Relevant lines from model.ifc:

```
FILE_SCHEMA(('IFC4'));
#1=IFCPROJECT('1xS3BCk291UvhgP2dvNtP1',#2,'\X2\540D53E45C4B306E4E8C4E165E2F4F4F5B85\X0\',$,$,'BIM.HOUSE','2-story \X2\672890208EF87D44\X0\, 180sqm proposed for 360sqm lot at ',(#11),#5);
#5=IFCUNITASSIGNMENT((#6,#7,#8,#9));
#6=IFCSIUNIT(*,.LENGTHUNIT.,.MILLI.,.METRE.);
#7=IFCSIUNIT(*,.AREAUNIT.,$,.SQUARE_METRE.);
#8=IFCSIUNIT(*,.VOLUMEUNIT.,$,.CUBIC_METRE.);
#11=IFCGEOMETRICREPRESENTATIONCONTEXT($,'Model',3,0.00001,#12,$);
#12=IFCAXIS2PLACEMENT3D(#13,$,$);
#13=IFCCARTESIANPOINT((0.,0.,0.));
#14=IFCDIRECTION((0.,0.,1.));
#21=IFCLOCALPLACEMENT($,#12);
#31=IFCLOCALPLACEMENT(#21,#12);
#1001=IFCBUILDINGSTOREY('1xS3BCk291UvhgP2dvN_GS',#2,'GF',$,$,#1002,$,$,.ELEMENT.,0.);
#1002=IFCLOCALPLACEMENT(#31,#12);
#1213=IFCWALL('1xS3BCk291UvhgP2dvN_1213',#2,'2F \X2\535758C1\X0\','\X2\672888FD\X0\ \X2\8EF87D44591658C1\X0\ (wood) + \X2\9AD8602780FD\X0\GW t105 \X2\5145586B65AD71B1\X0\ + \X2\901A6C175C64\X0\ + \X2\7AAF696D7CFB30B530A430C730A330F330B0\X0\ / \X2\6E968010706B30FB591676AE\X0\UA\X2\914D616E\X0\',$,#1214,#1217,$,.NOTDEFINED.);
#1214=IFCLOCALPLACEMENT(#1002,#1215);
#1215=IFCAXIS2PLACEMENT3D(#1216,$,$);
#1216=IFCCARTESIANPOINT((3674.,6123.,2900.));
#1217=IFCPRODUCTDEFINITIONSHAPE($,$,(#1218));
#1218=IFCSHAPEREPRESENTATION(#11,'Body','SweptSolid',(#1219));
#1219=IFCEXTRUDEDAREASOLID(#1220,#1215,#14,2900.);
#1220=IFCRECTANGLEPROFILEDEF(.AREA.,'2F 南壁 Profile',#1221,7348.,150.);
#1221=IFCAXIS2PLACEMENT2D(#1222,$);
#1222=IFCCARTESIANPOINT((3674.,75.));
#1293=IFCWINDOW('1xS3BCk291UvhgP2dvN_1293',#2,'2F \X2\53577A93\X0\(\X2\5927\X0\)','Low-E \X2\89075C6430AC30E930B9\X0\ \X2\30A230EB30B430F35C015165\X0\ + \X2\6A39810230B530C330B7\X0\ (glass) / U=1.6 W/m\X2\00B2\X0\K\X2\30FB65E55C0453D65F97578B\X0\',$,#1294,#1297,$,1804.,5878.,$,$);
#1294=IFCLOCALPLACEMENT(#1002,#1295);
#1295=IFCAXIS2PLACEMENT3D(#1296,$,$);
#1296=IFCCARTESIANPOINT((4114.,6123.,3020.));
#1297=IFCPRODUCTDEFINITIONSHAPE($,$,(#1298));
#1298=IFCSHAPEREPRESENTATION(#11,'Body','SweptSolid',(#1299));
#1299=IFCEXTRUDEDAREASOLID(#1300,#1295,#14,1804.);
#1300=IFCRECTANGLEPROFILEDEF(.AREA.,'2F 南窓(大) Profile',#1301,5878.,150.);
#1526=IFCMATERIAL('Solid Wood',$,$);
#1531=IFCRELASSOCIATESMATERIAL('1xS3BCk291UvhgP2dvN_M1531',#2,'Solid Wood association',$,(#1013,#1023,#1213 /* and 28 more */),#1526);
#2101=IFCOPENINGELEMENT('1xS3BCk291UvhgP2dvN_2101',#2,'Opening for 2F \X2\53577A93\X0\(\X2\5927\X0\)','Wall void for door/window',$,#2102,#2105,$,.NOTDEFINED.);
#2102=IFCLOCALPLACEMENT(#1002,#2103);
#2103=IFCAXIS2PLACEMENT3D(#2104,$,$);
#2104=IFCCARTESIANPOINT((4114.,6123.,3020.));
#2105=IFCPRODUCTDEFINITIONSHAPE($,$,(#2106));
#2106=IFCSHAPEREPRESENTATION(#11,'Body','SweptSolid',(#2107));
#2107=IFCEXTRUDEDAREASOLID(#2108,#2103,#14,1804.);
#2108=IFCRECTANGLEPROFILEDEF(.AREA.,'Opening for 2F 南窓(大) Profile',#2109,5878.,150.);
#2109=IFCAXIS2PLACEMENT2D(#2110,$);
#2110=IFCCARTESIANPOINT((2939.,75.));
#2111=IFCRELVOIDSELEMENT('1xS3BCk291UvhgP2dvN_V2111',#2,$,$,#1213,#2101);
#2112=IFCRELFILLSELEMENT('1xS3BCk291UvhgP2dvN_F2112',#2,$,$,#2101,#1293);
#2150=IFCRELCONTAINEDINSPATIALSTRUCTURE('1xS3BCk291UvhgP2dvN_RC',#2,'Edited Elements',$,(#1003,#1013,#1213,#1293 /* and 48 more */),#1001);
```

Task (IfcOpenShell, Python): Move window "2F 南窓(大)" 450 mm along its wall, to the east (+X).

```python
import ifcopenshell
import ifcopenshell.api.geometry
import ifcopenshell.util.placement

model = ifcopenshell.open("model.ifc")

window = model.by_id(1293)
opening = window.FillsVoids[0].RelatingOpeningElement
wall = opening.VoidsElements[0].RelatingBuildingElement

wall_matrix = ifcopenshell.util.placement.get_local_placement(wall.ObjectPlacement)
shift = wall_matrix[:3, 0] * 450.0
before = ifcopenshell.util.placement.get_local_placement(window.ObjectPlacement)[:3, 3].copy()

# The window is not placed relative to its opening, so move both.
for product in (opening, window):
    matrix = ifcopenshell.util.placement.get_local_placement(product.ObjectPlacement)
    matrix[:3, 3] += shift
    ifcopenshell.api.geometry.edit_object_placement(model, product=product, matrix=matrix, is_si=False)

after = ifcopenshell.util.placement.get_local_placement(window.ObjectPlacement)[:3, 3]
print("window moved by", (after - before).round(3) + 0.0)

model.write("model_updated.ifc")
```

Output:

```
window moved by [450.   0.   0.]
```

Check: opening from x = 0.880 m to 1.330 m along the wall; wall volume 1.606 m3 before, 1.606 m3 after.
